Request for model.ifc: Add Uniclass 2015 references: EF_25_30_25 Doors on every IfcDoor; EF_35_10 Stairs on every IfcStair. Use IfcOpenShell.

First a look at what the model holds.

```python
import ifcopenshell

model = ifcopenshell.open("model.ifc")
print(model.schema)
print("classifications:", [c.Name for c in model.by_type("IfcClassification")])
for ifc_class in ("IfcDoor", "IfcRoof", "IfcStair", "IfcWall", "IfcWindow"):
    print(ifc_class, len(model.by_type(ifc_class)))
```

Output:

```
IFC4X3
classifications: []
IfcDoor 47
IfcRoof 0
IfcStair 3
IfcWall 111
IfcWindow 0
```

```python
import ifcopenshell
import ifcopenshell.api.classification

model = ifcopenshell.open("model.ifc")

system = ifcopenshell.api.classification.add_classification(model, classification="Uniclass 2015")

codes = {
    "IfcDoor": ("EF_25_30_25", "Doors"),
    "IfcStair": ("EF_35_10", "Stairs"),
}
for ifc_class, (code, name) in codes.items():
    products = model.by_type(ifc_class)
    ifcopenshell.api.classification.add_reference(
        model, products=products, classification=system, identification=code, name=name
    )
    print(code, len(products))

model.write("model-out.ifc")
```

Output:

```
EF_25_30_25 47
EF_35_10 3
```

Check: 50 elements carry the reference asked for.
